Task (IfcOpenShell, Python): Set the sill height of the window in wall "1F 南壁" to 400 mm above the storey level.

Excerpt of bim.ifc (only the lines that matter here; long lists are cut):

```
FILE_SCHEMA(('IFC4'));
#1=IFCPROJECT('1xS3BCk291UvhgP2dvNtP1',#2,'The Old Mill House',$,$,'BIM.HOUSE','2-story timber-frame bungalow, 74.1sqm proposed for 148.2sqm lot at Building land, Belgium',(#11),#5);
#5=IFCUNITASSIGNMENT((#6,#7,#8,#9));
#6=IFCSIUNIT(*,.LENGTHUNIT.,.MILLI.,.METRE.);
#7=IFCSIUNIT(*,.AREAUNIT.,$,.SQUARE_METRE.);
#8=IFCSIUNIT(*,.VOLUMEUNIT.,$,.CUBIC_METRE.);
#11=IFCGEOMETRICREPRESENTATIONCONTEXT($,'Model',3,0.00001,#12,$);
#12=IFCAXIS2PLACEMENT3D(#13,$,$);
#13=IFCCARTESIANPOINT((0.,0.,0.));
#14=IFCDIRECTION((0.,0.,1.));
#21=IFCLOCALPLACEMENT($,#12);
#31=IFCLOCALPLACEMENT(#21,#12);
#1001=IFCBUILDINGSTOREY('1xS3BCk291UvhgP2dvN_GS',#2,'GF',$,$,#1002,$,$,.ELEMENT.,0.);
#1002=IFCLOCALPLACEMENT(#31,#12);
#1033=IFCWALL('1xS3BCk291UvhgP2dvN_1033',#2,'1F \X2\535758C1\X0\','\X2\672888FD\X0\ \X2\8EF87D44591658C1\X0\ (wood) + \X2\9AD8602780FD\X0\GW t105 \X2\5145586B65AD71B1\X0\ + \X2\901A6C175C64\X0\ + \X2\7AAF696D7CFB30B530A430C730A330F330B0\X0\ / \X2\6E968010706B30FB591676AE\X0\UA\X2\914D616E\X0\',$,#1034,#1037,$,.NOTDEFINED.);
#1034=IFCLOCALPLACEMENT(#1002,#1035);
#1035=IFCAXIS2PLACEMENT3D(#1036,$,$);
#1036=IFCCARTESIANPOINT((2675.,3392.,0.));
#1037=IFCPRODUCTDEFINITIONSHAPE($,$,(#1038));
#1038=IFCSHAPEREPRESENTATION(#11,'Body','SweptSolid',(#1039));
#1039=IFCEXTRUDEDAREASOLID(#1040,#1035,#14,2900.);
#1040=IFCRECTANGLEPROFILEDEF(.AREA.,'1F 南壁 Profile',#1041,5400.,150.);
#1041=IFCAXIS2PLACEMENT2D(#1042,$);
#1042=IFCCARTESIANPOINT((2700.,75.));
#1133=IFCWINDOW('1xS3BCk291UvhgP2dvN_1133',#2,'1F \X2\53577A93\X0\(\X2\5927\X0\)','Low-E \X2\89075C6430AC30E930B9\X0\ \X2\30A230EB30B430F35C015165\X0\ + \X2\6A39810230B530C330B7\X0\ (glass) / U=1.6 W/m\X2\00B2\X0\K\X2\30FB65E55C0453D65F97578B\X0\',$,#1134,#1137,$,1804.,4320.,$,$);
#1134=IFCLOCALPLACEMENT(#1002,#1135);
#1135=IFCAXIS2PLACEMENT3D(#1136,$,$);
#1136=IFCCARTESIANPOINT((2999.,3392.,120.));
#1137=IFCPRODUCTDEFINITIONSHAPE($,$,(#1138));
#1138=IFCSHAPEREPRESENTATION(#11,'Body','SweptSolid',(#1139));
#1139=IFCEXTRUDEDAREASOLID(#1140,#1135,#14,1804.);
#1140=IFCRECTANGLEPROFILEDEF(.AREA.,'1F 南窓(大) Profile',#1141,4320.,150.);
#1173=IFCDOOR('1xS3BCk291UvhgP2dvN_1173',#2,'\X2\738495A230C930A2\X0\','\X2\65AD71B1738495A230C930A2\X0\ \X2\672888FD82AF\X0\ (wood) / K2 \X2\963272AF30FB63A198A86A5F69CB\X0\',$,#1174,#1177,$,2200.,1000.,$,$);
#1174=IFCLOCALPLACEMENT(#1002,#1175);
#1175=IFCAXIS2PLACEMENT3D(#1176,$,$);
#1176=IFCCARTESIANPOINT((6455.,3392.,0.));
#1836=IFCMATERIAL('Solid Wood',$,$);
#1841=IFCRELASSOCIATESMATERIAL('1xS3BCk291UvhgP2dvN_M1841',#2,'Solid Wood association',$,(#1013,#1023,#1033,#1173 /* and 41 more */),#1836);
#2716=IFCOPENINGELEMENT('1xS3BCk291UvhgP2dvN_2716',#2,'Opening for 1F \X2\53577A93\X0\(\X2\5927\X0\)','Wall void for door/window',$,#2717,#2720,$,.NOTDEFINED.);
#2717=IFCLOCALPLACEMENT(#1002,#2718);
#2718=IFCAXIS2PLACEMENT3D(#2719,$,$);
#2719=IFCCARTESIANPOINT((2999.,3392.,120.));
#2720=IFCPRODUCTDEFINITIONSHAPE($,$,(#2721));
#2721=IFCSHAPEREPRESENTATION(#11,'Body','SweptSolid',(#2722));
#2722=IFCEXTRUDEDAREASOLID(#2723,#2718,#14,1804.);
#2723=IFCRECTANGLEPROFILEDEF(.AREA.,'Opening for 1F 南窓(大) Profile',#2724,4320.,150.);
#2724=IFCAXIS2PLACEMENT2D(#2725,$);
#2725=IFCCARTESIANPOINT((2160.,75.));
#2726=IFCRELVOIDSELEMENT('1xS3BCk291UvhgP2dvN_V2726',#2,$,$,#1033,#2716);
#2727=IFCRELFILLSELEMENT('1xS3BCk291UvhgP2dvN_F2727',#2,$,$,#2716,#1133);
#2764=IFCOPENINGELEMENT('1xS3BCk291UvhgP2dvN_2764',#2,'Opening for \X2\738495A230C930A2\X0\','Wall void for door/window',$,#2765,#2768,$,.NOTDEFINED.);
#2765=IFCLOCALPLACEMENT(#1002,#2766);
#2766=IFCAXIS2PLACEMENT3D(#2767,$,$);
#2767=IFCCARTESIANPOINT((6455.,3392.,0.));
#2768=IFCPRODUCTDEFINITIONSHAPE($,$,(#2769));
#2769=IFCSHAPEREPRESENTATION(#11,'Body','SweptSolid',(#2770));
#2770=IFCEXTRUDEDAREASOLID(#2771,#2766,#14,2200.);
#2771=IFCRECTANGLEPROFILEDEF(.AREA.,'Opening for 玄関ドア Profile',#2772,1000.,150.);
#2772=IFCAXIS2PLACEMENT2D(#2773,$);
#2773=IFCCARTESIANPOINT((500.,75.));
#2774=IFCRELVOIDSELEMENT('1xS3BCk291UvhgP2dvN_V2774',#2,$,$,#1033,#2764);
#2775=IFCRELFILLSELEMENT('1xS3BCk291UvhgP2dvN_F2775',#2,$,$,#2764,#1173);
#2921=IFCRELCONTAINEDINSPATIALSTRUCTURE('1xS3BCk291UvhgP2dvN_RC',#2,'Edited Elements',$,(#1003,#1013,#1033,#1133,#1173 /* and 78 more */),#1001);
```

```python
import numpy as np
import ifcopenshell
import ifcopenshell.api.geometry
import ifcopenshell.geom
import ifcopenshell.util.element
import ifcopenshell.util.placement
import ifcopenshell.util.shape
import ifcopenshell.util.unit

model = ifcopenshell.open("bim.ifc")
unit_scale = ifcopenshell.util.unit.calculate_unit_scale(model)

window = model.by_id(1133)
opening = window.FillsVoids[0].RelatingOpeningElement
storey = ifcopenshell.util.element.get_container(window, ifc_class="IfcBuildingStorey")
level = ifcopenshell.util.placement.get_local_placement(storey.ObjectPlacement)[2, 3]

# The opening's origin need not be at the sill, so measure its lowest point.
shape = ifcopenshell.geom.create_shape(ifcopenshell.geom.settings(), opening)
bottom = ifcopenshell.util.shape.get_shape_bottom_elevation(shape, shape.geometry) / unit_scale
dz = level + 0.4 / unit_scale - bottom

shift = np.array([0.0, 0.0, dz])
# The window is not placed relative to its opening, so move both.
for product in (opening, window):
    matrix = ifcopenshell.util.placement.get_local_placement(product.ObjectPlacement)
    matrix[:3, 3] += shift
    ifcopenshell.api.geometry.edit_object_placement(model, product=product, matrix=matrix, is_si=False)

print(f"moved by {dz * unit_scale:+.3f} m")

model.write("bim_edited.ifc")
```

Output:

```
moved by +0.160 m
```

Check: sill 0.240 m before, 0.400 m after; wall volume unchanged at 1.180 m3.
